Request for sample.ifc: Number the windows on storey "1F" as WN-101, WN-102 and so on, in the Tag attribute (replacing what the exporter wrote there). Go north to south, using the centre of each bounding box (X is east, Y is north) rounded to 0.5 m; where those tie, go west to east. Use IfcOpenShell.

First a look at what the model holds.

```python
import ifcopenshell
import ifcopenshell.util.element
import ifcopenshell.util.placement

model = ifcopenshell.open("sample.ifc")
print(model.schema)
storey = next(s for s in model.by_type("IfcBuildingStorey") if s.Name == "1F")
windows = [e for e in ifcopenshell.util.element.get_decomposition(storey) if e.is_a("IfcWindow")]
for e in sorted(windows, key=lambda e: e.id()):
    origin = ifcopenshell.util.placement.get_local_placement(e.ObjectPlacement)[:3, 3]
    print(e.id(), e.Tag, e.Name, origin.round(2) + 0.0, sep=" | ")
```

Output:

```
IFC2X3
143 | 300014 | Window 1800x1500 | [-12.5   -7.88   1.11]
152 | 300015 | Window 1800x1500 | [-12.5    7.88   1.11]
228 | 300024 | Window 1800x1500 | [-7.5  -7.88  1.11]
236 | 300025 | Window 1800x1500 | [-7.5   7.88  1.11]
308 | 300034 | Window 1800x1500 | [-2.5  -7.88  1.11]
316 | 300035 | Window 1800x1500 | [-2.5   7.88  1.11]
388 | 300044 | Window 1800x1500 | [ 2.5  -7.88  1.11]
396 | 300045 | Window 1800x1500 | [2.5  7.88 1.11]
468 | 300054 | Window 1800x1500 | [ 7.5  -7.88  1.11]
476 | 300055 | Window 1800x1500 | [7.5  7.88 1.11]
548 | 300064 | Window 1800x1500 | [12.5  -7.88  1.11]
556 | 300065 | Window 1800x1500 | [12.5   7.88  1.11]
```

```python
import ifcopenshell
import ifcopenshell.geom
import ifcopenshell.util.element
import ifcopenshell.util.shape

model = ifcopenshell.open("sample.ifc")
settings = ifcopenshell.geom.settings()
settings.set("use-world-coords", True)


def centre(element):
    shape = ifcopenshell.geom.create_shape(settings, element)
    return ifcopenshell.util.shape.get_bbox_centroid(shape.geometry)


storey = next(s for s in model.by_type("IfcBuildingStorey") if s.Name == "1F")
windows = [e for e in ifcopenshell.util.element.get_decomposition(storey) if e.is_a("IfcWindow")]

# Insertion points can sit at a corner or the storey origin, so sort by the geometry (in metres).
centres = {e: centre(e) for e in windows}
windows.sort(key=lambda e: (-round(centres[e][1] / 0.5), centres[e][0]))

for i, e in enumerate(windows, start=1):
    number = f"WN-1{i:02d}"
    e.Tag = number
    print(e.id(), number)

model.write("sample_v2.ifc")
```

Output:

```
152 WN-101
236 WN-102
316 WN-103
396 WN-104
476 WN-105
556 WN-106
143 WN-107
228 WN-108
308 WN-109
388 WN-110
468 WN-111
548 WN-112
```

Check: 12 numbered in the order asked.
